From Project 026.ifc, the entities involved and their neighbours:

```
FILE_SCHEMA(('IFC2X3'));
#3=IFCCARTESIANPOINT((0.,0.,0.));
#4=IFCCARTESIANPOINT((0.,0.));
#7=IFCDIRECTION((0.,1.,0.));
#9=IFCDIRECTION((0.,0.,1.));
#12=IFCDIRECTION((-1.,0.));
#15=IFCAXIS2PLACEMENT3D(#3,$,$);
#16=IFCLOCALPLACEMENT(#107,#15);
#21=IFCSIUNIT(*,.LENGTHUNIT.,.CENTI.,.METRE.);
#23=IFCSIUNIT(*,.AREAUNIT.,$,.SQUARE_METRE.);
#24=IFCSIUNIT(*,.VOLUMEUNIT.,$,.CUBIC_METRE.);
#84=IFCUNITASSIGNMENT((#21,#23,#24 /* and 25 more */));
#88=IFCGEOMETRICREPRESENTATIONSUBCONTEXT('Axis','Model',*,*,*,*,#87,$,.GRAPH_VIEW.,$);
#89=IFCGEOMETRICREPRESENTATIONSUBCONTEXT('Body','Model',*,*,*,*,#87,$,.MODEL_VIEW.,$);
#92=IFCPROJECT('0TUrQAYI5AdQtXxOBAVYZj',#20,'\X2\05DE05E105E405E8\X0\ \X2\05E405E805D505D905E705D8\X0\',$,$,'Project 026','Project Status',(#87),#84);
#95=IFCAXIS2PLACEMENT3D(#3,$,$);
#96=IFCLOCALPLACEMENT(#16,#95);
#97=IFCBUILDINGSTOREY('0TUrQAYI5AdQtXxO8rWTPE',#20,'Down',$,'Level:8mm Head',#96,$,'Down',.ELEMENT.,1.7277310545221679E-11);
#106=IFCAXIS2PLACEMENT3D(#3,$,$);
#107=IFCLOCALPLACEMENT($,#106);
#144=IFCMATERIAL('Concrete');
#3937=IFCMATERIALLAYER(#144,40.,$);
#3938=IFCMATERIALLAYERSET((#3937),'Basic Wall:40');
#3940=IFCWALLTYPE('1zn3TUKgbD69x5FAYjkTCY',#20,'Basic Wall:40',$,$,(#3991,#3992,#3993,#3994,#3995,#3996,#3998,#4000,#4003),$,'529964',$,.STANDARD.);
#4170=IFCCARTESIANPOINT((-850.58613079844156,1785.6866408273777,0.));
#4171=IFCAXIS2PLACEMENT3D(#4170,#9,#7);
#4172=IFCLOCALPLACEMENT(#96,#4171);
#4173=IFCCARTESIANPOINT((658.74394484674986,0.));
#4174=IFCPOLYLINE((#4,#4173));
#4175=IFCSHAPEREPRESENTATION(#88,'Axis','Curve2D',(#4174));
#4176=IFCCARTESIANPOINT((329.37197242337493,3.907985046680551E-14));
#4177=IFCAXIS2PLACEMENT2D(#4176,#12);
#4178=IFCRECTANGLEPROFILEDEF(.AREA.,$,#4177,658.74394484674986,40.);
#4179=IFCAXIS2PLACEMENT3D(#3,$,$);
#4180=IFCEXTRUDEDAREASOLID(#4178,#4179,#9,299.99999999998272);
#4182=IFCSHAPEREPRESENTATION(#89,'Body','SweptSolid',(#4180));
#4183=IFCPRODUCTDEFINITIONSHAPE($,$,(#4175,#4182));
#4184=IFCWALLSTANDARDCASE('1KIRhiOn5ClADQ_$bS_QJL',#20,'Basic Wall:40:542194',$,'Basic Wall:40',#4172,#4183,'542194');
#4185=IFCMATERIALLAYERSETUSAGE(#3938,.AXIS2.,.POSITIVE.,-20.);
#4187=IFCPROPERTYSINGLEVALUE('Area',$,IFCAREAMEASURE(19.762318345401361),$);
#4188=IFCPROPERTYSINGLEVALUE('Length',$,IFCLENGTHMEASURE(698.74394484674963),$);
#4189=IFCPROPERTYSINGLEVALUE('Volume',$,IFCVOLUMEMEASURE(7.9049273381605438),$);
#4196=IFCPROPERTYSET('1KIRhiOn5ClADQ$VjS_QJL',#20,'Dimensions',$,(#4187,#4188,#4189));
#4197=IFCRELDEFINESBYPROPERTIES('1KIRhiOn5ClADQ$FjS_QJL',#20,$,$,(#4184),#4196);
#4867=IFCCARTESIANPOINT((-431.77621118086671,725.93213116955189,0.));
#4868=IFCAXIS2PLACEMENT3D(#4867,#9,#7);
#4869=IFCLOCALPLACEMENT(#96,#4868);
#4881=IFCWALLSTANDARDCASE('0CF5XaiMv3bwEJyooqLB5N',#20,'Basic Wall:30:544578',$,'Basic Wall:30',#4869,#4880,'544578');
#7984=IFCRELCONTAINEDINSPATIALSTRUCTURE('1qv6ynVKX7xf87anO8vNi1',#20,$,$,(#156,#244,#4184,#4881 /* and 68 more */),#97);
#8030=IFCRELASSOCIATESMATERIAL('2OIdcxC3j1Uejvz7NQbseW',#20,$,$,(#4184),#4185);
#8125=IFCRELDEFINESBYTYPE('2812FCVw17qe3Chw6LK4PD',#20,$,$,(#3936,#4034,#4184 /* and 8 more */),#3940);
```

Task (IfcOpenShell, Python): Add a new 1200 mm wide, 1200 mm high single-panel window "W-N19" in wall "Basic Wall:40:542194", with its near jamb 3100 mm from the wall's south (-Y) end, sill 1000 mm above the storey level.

```python
import numpy as np
import ifcopenshell
import ifcopenshell.api.feature
import ifcopenshell.api.geometry
import ifcopenshell.api.pset
import ifcopenshell.api.root
import ifcopenshell.api.spatial
import ifcopenshell.api.type
import ifcopenshell.geom
import ifcopenshell.util.element
import ifcopenshell.util.placement
import ifcopenshell.util.representation
import ifcopenshell.util.shape
import ifcopenshell.util.unit

model = ifcopenshell.open("Project 026.ifc")
unit_scale = ifcopenshell.util.unit.calculate_unit_scale(model)
area_scale = ifcopenshell.util.unit.calculate_unit_scale(model, "AREAUNIT")
volume_scale = ifcopenshell.util.unit.calculate_unit_scale(model, "VOLUMEUNIT")
settings = ifcopenshell.geom.settings()


def volume(element):
    """Net volume in cubic metres, openings subtracted."""
    shape = ifcopenshell.geom.create_shape(settings, element)
    return ifcopenshell.util.shape.get_volume(shape.geometry)


wall = model.by_id(4184)
storey = ifcopenshell.util.element.get_container(wall, ifc_class="IfcBuildingStorey")
context = ifcopenshell.util.representation.get_context(model, "Model", "Body", "MODEL_VIEW")
before = volume(wall)

width, height, from_end, sill = 1.2, 1.2, 3.1, 1  # metres

# The wall runs along its own X axis, and the end named is its -X end.
wall_shape = ifcopenshell.geom.create_shape(settings, wall)
x, y, z = ifcopenshell.util.shape.get_vertices(wall_shape.geometry).T
start = x.min() + from_end
face, thickness = float(y.min()), float(y.max() - y.min())
wall_matrix = ifcopenshell.util.placement.get_local_placement(wall.ObjectPlacement)
level = ifcopenshell.util.placement.get_local_placement(storey.ObjectPlacement)[2, 3]


def in_wall(x, y):
    """Placement at x, y metres in the wall's axes, at sill height."""
    matrix = wall_matrix.copy()
    matrix[:, 3] = wall_matrix @ np.array([x / unit_scale, y / unit_scale, 0.0, 1.0])
    matrix[2, 3] = level + sill / unit_scale
    return matrix


# Opening: a box that overshoots both wall faces by 50 mm.
opening = ifcopenshell.api.root.create_entity(model, ifc_class="IfcOpeningElement")
box = ifcopenshell.api.geometry.add_wall_representation(
    model, context=context, length=width, height=height, thickness=thickness + 0.1
)
ifcopenshell.api.geometry.assign_representation(model, product=opening, representation=box)
ifcopenshell.api.geometry.edit_object_placement(model, product=opening, matrix=in_wall(start, face - 0.05), is_si=False)
ifcopenshell.api.feature.add_feature(model, feature=opening, element=wall)

window = ifcopenshell.api.root.create_entity(model, ifc_class="IfcWindow", name="W-N19")
window.OverallWidth, window.OverallHeight = width / unit_scale, height / unit_scale
body = ifcopenshell.api.geometry.add_window_representation(
    model,
    context=context,
    overall_width=window.OverallWidth,
    overall_height=window.OverallHeight,
    partition_type="SINGLE_PANEL",
)
ifcopenshell.api.geometry.assign_representation(model, product=window, representation=body)
ifcopenshell.api.spatial.assign_container(model, products=[window], relating_structure=storey)
fills = ifcopenshell.api.feature.add_filling(model, opening=opening, element=window)
fills.OwnerHistory = window.OwnerHistory  # required in IFC2X3

# IFC2X3 keeps the operation on the window style.
style = ifcopenshell.api.root.create_entity(model, ifc_class="IfcWindowStyle", name="W-N19")
style.OperationType, style.ConstructionType = "SINGLE_PANEL", "NOTDEFINED"
style.ParameterTakesPrecedence = style.Sizeable = False
ifcopenshell.api.type.assign_type(model, related_objects=[window], relating_type=style)

# Centre the window in the wall's thickness.
ifcopenshell.api.geometry.edit_object_placement(model, product=window, matrix=in_wall(start, face), is_si=False)
window_shape = ifcopenshell.geom.create_shape(settings, window)
depth = ifcopenshell.util.shape.get_vertices(window_shape.geometry)[:, 1]
offset = face + thickness / 2 - (depth.min() + depth.max()) / 2
ifcopenshell.api.geometry.edit_object_placement(model, product=window, matrix=in_wall(start, offset), is_si=False)

after = volume(wall)

# Update the wall's stored quantities.
pset = model.by_id(ifcopenshell.util.element.get_pset(wall, "Dimensions", should_inherit=False)["id"])
ifcopenshell.api.pset.edit_pset(model, pset=pset, properties={
    "Area": model.create_entity("IfcAreaMeasure", after / thickness / area_scale),
    "Volume": model.create_entity("IfcVolumeMeasure", after / volume_scale),
})

print(f"wall volume {before:.3f} -> {after:.3f} m3")

model.write("Project 026-out.ifc")
```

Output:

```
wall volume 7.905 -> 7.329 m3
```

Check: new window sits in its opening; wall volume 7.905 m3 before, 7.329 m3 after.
